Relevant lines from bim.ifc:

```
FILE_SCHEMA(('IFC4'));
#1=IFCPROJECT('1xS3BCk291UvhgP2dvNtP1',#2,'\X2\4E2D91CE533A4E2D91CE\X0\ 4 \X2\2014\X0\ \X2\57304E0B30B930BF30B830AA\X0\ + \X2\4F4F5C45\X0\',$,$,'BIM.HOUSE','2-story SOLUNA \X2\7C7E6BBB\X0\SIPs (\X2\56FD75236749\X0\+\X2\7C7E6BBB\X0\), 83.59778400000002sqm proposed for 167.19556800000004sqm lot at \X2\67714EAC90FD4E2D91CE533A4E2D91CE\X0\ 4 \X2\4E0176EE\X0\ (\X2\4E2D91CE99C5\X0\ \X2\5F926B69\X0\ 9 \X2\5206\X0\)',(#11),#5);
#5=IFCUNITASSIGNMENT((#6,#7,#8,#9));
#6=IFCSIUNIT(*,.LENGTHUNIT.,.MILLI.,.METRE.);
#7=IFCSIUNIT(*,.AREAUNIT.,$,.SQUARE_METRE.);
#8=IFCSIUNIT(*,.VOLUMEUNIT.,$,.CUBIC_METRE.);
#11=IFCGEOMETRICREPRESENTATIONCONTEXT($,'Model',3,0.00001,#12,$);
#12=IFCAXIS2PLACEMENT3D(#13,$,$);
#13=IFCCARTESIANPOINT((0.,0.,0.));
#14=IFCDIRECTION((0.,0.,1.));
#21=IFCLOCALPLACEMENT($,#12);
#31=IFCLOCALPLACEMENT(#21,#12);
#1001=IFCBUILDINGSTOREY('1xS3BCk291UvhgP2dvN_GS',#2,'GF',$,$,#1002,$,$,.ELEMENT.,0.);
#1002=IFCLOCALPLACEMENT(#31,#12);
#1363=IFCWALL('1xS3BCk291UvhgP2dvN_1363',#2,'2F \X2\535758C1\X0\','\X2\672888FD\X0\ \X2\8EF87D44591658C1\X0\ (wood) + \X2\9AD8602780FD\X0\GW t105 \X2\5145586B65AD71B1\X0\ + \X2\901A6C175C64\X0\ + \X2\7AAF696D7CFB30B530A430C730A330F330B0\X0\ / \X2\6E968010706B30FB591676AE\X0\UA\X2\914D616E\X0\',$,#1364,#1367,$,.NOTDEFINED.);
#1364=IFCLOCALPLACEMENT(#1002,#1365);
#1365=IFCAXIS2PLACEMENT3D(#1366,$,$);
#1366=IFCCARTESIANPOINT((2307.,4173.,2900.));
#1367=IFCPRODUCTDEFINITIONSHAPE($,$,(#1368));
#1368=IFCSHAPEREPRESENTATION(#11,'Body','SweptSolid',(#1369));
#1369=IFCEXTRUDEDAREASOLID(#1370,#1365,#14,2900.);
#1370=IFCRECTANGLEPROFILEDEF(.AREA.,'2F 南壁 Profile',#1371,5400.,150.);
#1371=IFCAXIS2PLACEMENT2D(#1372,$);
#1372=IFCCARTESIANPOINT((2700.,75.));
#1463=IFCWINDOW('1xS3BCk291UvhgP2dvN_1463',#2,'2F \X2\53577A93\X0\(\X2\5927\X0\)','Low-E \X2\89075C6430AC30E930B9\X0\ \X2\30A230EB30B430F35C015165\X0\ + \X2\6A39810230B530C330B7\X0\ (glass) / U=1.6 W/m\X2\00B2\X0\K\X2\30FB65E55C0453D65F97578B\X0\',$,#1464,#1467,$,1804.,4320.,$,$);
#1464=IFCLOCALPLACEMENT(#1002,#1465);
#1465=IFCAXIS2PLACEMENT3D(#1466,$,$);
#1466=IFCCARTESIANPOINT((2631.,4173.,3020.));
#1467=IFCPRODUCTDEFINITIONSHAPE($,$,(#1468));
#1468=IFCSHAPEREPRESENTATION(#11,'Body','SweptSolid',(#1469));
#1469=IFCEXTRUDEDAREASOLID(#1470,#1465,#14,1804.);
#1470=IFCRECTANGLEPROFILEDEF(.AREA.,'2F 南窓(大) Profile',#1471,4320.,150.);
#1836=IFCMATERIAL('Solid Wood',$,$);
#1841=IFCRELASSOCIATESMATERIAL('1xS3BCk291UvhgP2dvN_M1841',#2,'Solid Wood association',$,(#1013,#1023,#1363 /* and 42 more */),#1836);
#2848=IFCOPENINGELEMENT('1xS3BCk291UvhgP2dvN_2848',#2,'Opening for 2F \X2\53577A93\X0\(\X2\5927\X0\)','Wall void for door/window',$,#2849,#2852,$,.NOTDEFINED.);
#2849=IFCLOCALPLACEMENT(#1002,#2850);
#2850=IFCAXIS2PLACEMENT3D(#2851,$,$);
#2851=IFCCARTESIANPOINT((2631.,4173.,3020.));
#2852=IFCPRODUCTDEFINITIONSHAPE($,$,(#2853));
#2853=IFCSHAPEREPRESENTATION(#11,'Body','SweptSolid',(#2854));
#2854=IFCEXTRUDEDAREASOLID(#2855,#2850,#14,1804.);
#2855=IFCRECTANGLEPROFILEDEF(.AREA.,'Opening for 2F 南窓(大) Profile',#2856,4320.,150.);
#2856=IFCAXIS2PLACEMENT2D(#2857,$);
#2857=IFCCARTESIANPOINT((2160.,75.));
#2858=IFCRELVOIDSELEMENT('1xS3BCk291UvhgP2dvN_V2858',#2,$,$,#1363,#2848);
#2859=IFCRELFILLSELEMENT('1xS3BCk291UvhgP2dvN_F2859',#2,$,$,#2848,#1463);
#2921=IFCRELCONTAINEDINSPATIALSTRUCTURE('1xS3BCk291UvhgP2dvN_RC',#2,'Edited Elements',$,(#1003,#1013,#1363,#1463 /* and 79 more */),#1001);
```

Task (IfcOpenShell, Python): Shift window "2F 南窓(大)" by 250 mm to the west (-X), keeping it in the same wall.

```python
import ifcopenshell
import ifcopenshell.api.geometry
import ifcopenshell.util.placement
import ifcopenshell.util.unit

model = ifcopenshell.open("bim.ifc")
unit_scale = ifcopenshell.util.unit.calculate_unit_scale(model)

window = model.by_guid("1xS3BCk291UvhgP2dvN_1463")
opening = window.FillsVoids[0].RelatingOpeningElement
wall = opening.VoidsElements[0].RelatingBuildingElement

wall_matrix = ifcopenshell.util.placement.get_local_placement(wall.ObjectPlacement)
shift = wall_matrix[:3, 0] * -0.25 / unit_scale
before = ifcopenshell.util.placement.get_local_placement(window.ObjectPlacement)[:3, 3].copy()

# The window is not placed relative to its opening, so move both.
for product in (opening, window):
    matrix = ifcopenshell.util.placement.get_local_placement(product.ObjectPlacement)
    matrix[:3, 3] += shift
    ifcopenshell.api.geometry.edit_object_placement(model, product=product, matrix=matrix, is_si=False)

after = ifcopenshell.util.placement.get_local_placement(window.ObjectPlacement)[:3, 3]
print("window moved by", (after - before).round(3) + 0.0)

model.write("bim_updated.ifc")
```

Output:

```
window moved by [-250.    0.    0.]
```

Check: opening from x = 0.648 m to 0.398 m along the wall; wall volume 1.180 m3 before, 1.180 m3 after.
